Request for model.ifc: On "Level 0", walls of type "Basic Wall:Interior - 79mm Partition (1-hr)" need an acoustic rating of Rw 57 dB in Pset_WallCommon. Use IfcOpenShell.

First a look at what the model holds.

```python
import ifcopenshell
import ifcopenshell.util.element

model = ifcopenshell.open("model.ifc")
print(model.schema)
storey = next(s for s in model.by_type("IfcBuildingStorey") if s.Name == "Level 0")
walls = [e for e in ifcopenshell.util.element.get_decomposition(storey) if e.is_a("IfcWall")]
seen = {}
for e in walls:
    element_type = ifcopenshell.util.element.get_type(e)
    key = (element_type.Name if element_type != e and element_type else None, ifcopenshell.util.element.get_pset(e, "Pset_WallCommon", "AcousticRating"))
    seen[key] = seen.get(key, 0) + 1
for (name, value), count in sorted(seen.items(), key=str):
    print(count, "x", name, "|", value)
```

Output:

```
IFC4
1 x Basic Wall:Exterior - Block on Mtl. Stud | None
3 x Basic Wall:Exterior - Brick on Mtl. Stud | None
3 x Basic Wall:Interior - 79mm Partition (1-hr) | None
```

```python
import ifcopenshell
import ifcopenshell.api.pset
import ifcopenshell.util.element

model = ifcopenshell.open("model.ifc")

storey = next(s for s in model.by_type("IfcBuildingStorey") if s.Name == "Level 0")
walls = [e for e in ifcopenshell.util.element.get_decomposition(storey) if e.is_a("IfcWall")]

count = 0
for e in walls:
    element_type = ifcopenshell.util.element.get_type(e)
    if element_type in (None, e) or element_type.Name != "Basic Wall:Interior - 79mm Partition (1-hr)":
        continue
    # add_pset returns the element's existing set when there is one.
    pset = ifcopenshell.api.pset.add_pset(model, product=e, name="Pset_WallCommon")
    ifcopenshell.api.pset.edit_pset(model, pset=pset, properties={"AcousticRating": "Rw 57 dB"})
    count += 1

print(count, "walls updated")

model.write("model_rev.ifc")
```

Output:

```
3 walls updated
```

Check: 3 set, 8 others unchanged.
